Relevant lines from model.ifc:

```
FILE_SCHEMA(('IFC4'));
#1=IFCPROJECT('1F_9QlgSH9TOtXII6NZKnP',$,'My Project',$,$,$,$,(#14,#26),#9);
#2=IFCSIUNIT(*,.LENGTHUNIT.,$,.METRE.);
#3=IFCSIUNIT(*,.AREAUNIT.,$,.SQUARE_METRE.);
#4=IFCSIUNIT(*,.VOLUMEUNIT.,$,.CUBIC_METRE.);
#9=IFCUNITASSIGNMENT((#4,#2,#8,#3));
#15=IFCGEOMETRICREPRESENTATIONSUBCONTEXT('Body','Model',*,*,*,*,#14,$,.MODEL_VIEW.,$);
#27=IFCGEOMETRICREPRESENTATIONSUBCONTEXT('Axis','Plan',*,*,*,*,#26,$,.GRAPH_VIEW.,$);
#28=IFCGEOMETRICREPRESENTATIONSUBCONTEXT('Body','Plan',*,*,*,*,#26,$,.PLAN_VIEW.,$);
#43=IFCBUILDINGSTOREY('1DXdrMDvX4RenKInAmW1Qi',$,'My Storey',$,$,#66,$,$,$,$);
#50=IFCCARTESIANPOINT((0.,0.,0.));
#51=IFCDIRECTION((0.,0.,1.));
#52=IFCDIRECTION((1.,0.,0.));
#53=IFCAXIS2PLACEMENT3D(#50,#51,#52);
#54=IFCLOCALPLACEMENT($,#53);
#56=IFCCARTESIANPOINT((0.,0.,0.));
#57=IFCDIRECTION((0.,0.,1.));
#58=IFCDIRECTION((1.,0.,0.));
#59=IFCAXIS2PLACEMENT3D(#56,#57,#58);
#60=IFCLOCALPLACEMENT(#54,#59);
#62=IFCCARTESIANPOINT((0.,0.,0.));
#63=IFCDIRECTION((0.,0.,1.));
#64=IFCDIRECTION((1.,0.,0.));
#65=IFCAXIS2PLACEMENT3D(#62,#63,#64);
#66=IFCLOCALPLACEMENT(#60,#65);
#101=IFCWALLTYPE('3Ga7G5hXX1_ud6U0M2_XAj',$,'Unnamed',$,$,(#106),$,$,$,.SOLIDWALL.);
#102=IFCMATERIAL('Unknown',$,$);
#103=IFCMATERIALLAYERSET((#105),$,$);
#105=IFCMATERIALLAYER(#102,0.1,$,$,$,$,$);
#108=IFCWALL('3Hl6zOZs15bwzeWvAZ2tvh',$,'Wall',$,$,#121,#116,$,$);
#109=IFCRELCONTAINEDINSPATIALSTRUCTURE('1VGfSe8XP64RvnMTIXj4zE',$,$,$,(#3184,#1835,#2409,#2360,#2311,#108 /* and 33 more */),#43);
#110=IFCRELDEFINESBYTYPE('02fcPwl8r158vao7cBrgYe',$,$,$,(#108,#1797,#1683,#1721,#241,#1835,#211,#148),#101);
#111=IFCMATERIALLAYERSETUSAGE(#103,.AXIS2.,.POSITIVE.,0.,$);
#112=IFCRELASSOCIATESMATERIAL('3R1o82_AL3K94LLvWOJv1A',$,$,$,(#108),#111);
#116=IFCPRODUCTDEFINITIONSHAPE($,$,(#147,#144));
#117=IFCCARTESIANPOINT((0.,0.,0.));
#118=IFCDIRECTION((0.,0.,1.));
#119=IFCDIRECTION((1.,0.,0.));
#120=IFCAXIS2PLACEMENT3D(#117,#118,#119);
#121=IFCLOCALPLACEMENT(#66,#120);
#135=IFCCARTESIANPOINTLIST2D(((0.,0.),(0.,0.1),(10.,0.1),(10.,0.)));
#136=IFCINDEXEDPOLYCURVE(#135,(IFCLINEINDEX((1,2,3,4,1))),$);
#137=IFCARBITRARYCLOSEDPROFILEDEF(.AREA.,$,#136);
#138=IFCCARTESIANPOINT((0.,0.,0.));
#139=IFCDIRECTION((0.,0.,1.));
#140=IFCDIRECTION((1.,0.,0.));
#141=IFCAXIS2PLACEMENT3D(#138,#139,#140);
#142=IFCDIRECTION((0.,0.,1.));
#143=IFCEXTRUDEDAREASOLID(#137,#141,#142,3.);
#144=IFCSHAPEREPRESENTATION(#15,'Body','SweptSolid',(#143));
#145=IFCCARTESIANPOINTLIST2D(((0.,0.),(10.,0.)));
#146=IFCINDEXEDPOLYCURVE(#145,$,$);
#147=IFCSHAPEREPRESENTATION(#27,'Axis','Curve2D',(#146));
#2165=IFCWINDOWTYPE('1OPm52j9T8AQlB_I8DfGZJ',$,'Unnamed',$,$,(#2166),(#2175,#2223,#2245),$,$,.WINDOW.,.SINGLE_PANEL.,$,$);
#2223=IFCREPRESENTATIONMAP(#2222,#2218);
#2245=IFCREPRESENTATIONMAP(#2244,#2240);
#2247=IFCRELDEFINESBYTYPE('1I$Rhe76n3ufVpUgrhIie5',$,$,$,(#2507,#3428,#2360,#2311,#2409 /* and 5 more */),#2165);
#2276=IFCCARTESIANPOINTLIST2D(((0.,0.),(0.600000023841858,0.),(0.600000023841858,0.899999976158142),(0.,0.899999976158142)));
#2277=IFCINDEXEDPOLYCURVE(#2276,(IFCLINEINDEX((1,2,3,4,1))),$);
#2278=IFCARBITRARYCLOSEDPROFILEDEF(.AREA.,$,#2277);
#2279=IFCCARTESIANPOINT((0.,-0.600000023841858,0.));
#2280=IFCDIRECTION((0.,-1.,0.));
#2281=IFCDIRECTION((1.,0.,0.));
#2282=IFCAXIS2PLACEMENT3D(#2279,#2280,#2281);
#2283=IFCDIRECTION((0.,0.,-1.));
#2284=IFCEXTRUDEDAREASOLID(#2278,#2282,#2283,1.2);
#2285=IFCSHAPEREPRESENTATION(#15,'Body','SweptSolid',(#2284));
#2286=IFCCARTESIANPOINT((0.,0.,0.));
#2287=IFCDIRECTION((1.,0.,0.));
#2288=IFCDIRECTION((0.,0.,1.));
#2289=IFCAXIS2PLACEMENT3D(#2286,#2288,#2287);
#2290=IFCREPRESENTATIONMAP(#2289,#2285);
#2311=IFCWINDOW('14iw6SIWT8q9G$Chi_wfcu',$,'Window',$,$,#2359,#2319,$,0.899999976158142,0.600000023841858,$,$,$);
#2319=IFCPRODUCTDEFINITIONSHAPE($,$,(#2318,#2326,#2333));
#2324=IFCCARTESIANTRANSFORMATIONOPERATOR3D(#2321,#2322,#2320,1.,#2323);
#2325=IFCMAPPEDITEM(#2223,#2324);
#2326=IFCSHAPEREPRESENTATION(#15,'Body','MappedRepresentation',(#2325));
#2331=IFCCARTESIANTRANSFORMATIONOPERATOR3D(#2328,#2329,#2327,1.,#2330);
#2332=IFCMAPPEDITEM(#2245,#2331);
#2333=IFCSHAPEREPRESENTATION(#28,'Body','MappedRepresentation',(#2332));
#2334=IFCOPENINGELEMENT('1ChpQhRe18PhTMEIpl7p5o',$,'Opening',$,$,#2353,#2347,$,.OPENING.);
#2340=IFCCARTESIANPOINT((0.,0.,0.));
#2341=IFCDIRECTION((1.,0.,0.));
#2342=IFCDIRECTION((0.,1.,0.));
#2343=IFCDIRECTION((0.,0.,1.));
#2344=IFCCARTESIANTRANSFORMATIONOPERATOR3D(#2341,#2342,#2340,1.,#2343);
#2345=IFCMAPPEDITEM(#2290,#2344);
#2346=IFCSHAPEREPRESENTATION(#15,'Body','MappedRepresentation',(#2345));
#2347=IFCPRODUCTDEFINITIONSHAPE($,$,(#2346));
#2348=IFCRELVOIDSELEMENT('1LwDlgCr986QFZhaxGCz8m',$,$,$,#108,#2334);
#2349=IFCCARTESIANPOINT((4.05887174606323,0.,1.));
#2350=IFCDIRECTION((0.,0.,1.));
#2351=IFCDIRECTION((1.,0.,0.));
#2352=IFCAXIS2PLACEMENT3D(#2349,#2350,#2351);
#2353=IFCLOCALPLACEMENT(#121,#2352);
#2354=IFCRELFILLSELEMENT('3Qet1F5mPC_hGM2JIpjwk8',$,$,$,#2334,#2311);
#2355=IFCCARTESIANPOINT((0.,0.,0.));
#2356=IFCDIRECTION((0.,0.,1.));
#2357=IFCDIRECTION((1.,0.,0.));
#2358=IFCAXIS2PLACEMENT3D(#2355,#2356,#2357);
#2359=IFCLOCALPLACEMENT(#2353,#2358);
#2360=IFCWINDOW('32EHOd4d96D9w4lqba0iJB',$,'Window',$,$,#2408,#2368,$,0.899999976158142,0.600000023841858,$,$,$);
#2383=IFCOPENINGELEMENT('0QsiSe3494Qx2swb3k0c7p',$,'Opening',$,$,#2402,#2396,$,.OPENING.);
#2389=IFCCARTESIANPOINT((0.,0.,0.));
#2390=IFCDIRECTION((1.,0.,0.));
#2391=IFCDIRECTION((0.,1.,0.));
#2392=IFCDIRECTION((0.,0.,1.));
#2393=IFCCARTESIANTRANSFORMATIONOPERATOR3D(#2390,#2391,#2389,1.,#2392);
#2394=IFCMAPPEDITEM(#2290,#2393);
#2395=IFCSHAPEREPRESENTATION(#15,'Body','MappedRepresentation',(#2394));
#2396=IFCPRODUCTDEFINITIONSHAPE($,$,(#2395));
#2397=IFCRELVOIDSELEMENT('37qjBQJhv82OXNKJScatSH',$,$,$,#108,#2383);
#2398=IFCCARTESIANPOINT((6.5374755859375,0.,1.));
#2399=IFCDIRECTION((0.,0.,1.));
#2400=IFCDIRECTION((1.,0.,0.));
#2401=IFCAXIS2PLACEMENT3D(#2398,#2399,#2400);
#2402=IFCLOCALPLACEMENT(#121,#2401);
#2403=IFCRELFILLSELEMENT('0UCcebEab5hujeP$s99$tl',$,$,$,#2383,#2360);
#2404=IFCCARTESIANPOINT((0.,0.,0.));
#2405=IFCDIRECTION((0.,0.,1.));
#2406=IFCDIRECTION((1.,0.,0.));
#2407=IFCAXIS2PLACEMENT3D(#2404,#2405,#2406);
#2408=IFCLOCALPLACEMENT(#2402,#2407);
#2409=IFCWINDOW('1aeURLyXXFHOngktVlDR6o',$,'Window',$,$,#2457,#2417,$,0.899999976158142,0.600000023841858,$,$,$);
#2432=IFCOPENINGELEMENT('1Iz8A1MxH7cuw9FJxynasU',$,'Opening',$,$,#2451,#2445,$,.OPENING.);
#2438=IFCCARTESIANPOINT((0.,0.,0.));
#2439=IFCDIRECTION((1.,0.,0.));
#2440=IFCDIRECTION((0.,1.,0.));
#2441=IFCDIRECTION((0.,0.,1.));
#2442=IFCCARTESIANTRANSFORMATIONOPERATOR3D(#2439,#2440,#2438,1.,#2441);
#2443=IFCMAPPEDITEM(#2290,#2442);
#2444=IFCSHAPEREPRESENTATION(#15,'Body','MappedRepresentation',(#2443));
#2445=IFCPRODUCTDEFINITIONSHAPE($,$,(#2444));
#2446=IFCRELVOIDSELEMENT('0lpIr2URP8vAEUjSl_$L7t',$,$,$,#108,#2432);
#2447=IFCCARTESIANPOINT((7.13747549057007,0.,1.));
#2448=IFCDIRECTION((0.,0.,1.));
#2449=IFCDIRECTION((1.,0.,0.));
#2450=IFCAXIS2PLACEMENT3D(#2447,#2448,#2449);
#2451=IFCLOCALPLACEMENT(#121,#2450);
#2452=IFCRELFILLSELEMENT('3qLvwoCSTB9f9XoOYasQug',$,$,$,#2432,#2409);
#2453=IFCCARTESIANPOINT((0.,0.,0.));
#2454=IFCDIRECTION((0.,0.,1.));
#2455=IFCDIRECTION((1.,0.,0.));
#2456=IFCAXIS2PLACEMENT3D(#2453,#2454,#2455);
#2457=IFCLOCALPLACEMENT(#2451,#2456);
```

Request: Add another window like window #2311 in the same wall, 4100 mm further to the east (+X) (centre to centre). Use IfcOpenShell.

```python
import ifcopenshell
import ifcopenshell.api.feature
import ifcopenshell.api.geometry
import ifcopenshell.api.root
import ifcopenshell.geom
import ifcopenshell.util.element
import ifcopenshell.util.placement
import ifcopenshell.util.shape
import ifcopenshell.util.unit

model = ifcopenshell.open("model.ifc")
unit_scale = ifcopenshell.util.unit.calculate_unit_scale(model)
settings = ifcopenshell.geom.settings()


def volume(element):
    """Net volume in cubic metres, openings subtracted."""
    shape = ifcopenshell.geom.create_shape(settings, element)
    return ifcopenshell.util.shape.get_volume(shape.geometry)


window = model.by_guid("14iw6SIWT8q9G$Chi_wfcu")
opening = window.FillsVoids[0].RelatingOpeningElement
wall = opening.VoidsElements[0].RelatingBuildingElement
before = volume(wall)
shift = ifcopenshell.util.placement.get_local_placement(wall.ObjectPlacement)[:3, 0] * 4.1 / unit_scale

# copy_class copies the void relationship, type, container and properties, but no geometry.
new_opening = ifcopenshell.api.root.copy_class(model, product=opening)
new_opening.Representation = ifcopenshell.util.element.copy_deep(
    model, opening.Representation, exclude=["IfcGeometricRepresentationContext", "IfcRepresentationMap"]
)
new_window = ifcopenshell.api.root.copy_class(model, product=window)
new_window.Representation = ifcopenshell.util.element.copy_deep(
    model, window.Representation, exclude=["IfcGeometricRepresentationContext", "IfcRepresentationMap"]
)
ifcopenshell.api.feature.add_filling(model, opening=new_opening, element=new_window)

for old, new in ((opening, new_opening), (window, new_window)):
    matrix = ifcopenshell.util.placement.get_local_placement(old.ObjectPlacement)
    matrix[:3, 3] += shift
    ifcopenshell.api.geometry.edit_object_placement(model, product=new, matrix=matrix, is_si=False)

after = volume(wall)

print(f"wall volume {before:.3f} -> {after:.3f} m3")

model.write("model_v2.ifc")
```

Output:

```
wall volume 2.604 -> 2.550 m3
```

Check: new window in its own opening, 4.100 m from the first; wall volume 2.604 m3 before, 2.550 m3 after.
